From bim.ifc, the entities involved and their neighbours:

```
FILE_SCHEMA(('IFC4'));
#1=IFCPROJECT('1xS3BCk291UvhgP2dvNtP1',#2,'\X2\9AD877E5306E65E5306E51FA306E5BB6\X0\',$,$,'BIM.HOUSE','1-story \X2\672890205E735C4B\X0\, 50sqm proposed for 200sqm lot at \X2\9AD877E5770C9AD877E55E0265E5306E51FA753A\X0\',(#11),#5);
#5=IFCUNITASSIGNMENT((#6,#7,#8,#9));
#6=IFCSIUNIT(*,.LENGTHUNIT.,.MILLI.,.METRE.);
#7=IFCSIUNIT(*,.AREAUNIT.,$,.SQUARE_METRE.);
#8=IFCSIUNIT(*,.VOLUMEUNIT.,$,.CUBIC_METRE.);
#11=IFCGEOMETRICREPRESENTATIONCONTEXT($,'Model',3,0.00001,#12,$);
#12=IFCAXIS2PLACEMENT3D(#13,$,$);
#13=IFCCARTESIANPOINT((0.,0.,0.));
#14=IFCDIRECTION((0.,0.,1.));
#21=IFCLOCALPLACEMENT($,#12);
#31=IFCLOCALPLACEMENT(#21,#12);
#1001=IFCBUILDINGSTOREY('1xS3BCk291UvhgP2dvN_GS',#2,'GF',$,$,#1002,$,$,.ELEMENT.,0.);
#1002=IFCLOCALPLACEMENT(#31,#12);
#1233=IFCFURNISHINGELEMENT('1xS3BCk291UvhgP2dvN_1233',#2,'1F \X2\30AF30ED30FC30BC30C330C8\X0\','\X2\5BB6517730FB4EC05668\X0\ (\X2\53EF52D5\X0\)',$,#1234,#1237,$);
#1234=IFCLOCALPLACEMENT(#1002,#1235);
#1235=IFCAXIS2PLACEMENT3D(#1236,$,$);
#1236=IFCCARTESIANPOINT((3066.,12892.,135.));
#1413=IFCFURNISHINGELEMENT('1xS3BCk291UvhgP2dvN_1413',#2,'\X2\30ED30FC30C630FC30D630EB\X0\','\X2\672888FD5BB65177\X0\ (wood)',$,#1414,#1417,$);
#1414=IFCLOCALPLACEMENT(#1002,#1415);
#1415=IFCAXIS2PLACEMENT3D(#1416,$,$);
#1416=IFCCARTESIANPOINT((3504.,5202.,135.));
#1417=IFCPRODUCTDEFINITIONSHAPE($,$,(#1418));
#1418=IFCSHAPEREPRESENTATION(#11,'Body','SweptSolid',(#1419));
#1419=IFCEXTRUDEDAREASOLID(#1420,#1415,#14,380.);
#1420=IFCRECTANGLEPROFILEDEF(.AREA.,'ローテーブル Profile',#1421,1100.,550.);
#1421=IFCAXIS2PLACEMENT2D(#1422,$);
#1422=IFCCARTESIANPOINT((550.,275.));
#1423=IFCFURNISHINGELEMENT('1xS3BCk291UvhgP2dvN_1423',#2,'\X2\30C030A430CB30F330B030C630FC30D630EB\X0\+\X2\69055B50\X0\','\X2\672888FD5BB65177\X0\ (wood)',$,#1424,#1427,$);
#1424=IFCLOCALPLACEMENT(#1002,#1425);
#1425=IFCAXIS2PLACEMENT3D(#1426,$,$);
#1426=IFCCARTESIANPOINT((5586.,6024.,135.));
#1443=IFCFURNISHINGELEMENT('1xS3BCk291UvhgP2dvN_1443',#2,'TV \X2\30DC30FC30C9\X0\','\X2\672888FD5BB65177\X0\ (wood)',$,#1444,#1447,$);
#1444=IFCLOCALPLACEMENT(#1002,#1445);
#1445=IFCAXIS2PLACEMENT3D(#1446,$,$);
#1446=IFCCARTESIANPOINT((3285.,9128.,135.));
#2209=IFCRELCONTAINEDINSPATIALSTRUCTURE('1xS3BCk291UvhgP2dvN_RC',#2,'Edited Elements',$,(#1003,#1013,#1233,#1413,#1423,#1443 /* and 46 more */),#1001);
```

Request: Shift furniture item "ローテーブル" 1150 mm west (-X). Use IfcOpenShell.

```python
import ifcopenshell
import ifcopenshell.api.geometry
import ifcopenshell.util.placement
import ifcopenshell.util.unit

model = ifcopenshell.open("bim.ifc")
unit_scale = ifcopenshell.util.unit.calculate_unit_scale(model)

item = model.by_guid("1xS3BCk291UvhgP2dvN_1413")
matrix = ifcopenshell.util.placement.get_local_placement(item.ObjectPlacement)
matrix[0, 3] -= 1.15 / unit_scale
ifcopenshell.api.geometry.edit_object_placement(model, product=item, matrix=matrix, is_si=False)

print(ifcopenshell.util.placement.get_local_placement(item.ObjectPlacement).round(3) + 0.0)

model.write("bim-out.ifc")
```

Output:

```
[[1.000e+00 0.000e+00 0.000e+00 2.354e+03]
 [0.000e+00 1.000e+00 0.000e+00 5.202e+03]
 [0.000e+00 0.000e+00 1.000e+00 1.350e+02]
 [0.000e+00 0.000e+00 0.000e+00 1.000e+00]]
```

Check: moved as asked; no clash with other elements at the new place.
